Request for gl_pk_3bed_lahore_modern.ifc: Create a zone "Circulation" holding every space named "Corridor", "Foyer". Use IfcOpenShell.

First a look at what the model holds.

```python
import ifcopenshell

model = ifcopenshell.open("gl_pk_3bed_lahore_modern.ifc")
print(model.schema)
seen = {}
for space in model.by_type("IfcSpace"):
    seen[space.LongName] = seen.get(space.LongName, 0) + 1
for name, count in sorted(seen.items(), key=str):
    print(count, "x", name)
print("zones:", [z.Name for z in model.by_type("IfcZone")][:20])
```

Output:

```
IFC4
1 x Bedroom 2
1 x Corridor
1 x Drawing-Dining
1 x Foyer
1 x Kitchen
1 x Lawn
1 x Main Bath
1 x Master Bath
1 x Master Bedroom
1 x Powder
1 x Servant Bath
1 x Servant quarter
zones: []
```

```python
import ifcopenshell
import ifcopenshell.api.group
import ifcopenshell.api.root

model = ifcopenshell.open("gl_pk_3bed_lahore_modern.ifc")

names = {"Corridor", "Foyer"}
spaces = [s for s in model.by_type("IfcSpace") if s.LongName in names]

zone = ifcopenshell.api.root.create_entity(model, ifc_class="IfcZone", name="Circulation")
ifcopenshell.api.group.assign_group(model, products=spaces, group=zone)
print(len(spaces), "spaces in", zone.Name)

model.write("gl_pk_3bed_lahore_modern-out.ifc")
```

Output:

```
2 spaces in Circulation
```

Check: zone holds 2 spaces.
